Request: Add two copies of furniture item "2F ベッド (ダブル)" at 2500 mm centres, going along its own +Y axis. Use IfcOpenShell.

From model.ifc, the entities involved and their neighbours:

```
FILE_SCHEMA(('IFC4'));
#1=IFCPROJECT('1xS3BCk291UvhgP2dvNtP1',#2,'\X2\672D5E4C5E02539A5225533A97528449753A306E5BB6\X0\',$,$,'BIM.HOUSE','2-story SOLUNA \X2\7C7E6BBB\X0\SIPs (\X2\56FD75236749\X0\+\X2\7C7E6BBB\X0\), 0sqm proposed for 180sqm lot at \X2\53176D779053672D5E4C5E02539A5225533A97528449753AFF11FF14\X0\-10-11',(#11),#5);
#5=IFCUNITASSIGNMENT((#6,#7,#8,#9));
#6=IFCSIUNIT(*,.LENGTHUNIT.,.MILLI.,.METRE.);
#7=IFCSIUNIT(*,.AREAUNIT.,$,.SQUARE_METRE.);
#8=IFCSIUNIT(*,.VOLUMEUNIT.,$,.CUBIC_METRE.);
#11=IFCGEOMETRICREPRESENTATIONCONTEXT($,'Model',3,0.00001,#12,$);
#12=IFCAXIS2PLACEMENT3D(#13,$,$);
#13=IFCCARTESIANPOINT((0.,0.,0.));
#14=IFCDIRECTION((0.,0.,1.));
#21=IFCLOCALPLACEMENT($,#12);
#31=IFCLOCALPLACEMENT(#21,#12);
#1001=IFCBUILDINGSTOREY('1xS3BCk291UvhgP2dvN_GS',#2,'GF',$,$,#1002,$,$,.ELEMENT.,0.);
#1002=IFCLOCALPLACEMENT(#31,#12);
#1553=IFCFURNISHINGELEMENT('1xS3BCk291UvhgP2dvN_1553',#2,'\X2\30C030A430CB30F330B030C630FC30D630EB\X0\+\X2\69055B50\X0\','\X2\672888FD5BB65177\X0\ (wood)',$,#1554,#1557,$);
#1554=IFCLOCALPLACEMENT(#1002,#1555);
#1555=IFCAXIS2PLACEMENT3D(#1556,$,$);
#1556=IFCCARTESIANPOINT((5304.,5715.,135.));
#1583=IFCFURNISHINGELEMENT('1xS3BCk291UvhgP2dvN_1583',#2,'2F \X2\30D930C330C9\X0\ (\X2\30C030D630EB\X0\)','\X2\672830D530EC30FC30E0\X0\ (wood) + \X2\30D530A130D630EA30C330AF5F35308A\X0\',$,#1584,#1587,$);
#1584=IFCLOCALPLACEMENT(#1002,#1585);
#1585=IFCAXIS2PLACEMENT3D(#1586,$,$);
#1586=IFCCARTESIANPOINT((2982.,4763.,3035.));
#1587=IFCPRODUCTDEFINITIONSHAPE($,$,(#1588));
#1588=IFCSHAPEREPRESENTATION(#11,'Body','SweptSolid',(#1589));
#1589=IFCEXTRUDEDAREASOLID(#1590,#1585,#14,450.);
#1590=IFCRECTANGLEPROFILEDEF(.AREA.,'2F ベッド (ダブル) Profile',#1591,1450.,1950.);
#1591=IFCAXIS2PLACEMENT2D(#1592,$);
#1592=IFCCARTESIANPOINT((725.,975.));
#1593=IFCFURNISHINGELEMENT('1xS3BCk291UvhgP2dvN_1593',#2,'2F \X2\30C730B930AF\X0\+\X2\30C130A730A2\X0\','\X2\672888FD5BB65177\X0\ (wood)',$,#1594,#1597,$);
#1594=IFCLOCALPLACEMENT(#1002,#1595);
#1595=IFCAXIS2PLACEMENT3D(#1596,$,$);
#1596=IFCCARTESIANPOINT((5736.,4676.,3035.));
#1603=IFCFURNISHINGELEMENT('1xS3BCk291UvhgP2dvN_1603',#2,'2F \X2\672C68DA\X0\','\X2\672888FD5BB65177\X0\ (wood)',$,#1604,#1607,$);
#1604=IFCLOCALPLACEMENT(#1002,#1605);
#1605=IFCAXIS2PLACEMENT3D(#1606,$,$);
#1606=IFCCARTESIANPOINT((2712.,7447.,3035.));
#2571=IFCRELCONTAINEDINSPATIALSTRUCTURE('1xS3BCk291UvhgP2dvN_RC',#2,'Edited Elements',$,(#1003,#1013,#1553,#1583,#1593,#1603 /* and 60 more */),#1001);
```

```python
import ifcopenshell
import ifcopenshell.api.geometry
import ifcopenshell.api.root
import ifcopenshell.util.element
import ifcopenshell.util.placement

model = ifcopenshell.open("model.ifc")


def reuse_history(source, copy):
    """copy_class also copies each property set's owner history, people and application; keep the originals."""
    for rel in copy.IsDefinedBy:
        if rel.is_a("IfcRelDefinesByProperties") and (history := rel.RelatingPropertyDefinition.OwnerHistory):
            rel.RelatingPropertyDefinition.OwnerHistory = source.OwnerHistory
            ifcopenshell.util.element.remove_deep2(model, history)


source = model.by_guid("1xS3BCk291UvhgP2dvN_1583")
base = ifcopenshell.util.placement.get_local_placement(source.ObjectPlacement)
step = base[:3, 1] * 2500.0

for i in range(1, 3):
    copy = ifcopenshell.api.root.copy_class(model, product=source)
    copy.Representation = ifcopenshell.util.element.copy_deep(
        model, source.Representation, exclude=["IfcGeometricRepresentationContext", "IfcRepresentationMap"]
    )
    reuse_history(source, copy)
    matrix = base.copy()
    matrix[:3, 3] += i * step
    print("added at", matrix[:3, 3].round(3) + 0.0)
    ifcopenshell.api.geometry.edit_object_placement(model, product=copy, matrix=matrix, is_si=False)

model.write("model_edited.ifc")
```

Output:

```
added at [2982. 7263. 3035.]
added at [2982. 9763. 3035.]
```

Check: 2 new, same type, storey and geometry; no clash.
